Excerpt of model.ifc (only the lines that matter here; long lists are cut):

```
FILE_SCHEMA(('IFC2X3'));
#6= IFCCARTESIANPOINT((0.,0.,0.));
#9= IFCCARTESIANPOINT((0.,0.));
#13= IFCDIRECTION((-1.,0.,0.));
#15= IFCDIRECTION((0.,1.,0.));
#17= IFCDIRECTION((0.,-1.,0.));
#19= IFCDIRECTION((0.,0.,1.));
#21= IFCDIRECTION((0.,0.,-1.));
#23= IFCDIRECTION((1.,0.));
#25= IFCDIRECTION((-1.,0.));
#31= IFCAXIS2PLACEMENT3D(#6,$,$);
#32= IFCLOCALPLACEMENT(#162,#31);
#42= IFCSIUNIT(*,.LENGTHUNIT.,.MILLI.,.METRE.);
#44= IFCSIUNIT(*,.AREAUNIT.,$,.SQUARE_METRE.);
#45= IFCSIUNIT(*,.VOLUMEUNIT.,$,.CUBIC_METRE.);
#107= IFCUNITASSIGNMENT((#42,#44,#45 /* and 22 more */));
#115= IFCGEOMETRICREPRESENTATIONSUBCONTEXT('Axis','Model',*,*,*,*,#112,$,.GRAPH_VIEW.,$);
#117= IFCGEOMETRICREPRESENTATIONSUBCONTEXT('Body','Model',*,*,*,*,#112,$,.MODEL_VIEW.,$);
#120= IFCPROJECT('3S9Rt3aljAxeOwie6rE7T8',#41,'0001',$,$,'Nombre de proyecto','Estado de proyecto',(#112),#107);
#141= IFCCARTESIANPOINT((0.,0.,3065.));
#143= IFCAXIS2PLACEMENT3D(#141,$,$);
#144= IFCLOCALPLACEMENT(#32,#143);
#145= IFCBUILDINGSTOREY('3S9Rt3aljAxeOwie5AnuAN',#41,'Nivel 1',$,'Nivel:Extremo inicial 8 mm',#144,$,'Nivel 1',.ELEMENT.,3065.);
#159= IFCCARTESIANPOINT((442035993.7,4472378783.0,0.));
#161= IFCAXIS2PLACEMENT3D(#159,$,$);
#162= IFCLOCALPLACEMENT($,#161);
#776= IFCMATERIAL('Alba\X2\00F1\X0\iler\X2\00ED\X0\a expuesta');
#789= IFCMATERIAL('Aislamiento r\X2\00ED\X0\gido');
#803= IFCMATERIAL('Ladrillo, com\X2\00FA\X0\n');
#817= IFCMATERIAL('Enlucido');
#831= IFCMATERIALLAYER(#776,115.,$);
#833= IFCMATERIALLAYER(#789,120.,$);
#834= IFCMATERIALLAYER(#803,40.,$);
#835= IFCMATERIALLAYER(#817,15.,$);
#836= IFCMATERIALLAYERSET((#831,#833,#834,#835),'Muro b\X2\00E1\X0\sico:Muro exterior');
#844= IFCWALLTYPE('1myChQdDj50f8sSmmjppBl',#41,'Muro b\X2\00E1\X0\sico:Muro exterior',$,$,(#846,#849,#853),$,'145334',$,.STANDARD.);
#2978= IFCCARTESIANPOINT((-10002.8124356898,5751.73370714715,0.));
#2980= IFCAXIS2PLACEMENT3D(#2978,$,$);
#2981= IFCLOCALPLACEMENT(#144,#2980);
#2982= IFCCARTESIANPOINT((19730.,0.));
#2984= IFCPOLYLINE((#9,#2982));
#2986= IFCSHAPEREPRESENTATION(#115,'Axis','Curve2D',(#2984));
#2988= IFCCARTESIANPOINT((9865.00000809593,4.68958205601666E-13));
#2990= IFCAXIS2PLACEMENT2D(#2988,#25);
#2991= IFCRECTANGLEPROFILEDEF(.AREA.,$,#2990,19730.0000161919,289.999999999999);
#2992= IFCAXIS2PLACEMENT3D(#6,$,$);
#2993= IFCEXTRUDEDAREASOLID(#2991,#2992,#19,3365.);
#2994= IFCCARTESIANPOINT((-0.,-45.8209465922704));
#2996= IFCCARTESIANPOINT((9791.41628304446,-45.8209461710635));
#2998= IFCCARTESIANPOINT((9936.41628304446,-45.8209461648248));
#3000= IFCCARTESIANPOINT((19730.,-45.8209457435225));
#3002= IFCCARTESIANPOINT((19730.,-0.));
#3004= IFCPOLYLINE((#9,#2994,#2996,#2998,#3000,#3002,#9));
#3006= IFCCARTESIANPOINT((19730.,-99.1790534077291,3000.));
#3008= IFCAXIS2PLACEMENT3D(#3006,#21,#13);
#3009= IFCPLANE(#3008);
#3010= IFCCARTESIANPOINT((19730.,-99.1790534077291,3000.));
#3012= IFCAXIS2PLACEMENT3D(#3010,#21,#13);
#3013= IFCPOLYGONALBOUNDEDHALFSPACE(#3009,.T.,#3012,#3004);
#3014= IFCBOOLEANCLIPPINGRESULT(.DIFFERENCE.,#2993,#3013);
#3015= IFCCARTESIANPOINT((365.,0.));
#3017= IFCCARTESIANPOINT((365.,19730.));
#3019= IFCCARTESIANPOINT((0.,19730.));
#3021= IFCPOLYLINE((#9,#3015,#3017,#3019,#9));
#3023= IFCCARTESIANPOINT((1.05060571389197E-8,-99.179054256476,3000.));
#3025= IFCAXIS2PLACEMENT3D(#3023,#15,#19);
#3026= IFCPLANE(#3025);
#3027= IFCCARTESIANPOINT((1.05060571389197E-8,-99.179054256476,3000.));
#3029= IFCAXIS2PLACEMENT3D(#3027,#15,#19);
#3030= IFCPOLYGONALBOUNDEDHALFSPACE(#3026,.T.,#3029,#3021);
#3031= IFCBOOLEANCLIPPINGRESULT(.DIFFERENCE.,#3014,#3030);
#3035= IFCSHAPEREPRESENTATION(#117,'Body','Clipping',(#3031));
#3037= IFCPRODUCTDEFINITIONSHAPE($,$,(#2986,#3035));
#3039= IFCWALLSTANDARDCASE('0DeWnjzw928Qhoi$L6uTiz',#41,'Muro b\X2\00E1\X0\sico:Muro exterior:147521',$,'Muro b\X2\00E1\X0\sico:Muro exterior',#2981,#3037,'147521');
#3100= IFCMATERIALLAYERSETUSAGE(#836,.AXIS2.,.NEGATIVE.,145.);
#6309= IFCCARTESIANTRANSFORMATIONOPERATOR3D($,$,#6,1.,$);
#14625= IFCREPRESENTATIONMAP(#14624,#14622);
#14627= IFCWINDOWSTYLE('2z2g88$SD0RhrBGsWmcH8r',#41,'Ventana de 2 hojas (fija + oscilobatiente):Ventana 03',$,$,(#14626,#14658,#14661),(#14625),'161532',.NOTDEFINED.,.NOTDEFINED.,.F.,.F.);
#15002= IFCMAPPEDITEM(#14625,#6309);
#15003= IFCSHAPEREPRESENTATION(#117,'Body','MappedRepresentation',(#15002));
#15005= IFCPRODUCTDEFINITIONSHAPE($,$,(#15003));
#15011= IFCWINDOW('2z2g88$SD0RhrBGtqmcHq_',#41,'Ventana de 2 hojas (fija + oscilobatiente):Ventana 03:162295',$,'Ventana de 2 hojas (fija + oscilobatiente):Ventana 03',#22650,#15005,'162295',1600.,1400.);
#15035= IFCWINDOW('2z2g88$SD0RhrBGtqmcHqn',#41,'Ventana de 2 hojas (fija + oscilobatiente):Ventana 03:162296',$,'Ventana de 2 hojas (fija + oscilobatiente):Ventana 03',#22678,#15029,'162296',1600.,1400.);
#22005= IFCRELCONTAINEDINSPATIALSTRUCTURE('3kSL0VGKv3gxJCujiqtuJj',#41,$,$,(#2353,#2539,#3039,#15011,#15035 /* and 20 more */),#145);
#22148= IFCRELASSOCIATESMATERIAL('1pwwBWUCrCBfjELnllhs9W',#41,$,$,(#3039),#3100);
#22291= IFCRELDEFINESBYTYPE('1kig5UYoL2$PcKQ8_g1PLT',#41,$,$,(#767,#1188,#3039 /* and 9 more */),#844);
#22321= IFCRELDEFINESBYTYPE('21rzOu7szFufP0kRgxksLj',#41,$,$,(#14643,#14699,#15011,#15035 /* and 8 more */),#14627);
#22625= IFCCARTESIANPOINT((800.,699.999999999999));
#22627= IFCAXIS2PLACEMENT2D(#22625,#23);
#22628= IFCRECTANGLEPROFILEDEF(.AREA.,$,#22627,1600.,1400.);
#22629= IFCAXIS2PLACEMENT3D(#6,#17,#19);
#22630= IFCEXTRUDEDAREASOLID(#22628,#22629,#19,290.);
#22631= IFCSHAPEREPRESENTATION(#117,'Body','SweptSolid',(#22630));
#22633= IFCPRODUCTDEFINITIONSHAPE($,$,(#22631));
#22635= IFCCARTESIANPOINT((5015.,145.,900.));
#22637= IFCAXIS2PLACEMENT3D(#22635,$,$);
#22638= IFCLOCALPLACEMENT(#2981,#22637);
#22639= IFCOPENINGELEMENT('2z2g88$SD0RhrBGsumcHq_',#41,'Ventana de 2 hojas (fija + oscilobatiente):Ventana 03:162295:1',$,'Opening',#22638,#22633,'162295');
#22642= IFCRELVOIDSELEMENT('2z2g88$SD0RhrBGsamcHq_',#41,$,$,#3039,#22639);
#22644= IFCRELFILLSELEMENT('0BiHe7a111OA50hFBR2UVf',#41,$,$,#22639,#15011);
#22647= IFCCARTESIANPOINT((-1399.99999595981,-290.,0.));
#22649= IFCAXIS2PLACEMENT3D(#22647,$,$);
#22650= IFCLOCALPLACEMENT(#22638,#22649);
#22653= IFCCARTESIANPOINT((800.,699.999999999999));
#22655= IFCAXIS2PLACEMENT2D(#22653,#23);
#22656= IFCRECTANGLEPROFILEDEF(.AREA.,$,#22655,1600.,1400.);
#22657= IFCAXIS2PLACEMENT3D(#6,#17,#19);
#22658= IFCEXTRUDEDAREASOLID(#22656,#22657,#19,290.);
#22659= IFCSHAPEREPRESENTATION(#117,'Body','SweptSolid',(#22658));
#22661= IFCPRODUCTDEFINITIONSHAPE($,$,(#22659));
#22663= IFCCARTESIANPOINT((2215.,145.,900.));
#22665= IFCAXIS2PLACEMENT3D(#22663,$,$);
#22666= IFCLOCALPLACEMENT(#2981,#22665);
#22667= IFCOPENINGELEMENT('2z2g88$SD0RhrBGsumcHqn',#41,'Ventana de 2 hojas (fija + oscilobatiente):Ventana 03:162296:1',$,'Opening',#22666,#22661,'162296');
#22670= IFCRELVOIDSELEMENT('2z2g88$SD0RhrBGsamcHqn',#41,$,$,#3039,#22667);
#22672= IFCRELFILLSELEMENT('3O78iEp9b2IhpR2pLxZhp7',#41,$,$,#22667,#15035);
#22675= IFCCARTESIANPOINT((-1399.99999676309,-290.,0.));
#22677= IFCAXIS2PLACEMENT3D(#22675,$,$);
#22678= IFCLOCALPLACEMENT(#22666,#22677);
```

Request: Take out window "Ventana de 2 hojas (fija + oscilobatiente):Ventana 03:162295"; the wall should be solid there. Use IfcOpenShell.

```python
import ifcopenshell
import ifcopenshell.api.feature
import ifcopenshell.api.root
import ifcopenshell.geom
import ifcopenshell.util.shape

model = ifcopenshell.open("model.ifc")
settings = ifcopenshell.geom.settings()


def volume(element):
    """Net volume in cubic metres, openings subtracted."""
    shape = ifcopenshell.geom.create_shape(settings, element)
    return ifcopenshell.util.shape.get_volume(shape.geometry)


window = model.by_guid("2z2g88$SD0RhrBGtqmcHq_")
opening = window.FillsVoids[0].RelatingOpeningElement
wall = opening.VoidsElements[0].RelatingBuildingElement
before = volume(wall)

ifcopenshell.api.root.remove_product(model, product=window)
ifcopenshell.api.feature.remove_feature(model, feature=opening)

after = volume(wall)

print(f"wall volume {before:.3f} -> {after:.3f} m3")

model.write("model-out.ifc")
```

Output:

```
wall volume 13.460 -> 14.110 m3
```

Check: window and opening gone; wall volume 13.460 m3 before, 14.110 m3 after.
